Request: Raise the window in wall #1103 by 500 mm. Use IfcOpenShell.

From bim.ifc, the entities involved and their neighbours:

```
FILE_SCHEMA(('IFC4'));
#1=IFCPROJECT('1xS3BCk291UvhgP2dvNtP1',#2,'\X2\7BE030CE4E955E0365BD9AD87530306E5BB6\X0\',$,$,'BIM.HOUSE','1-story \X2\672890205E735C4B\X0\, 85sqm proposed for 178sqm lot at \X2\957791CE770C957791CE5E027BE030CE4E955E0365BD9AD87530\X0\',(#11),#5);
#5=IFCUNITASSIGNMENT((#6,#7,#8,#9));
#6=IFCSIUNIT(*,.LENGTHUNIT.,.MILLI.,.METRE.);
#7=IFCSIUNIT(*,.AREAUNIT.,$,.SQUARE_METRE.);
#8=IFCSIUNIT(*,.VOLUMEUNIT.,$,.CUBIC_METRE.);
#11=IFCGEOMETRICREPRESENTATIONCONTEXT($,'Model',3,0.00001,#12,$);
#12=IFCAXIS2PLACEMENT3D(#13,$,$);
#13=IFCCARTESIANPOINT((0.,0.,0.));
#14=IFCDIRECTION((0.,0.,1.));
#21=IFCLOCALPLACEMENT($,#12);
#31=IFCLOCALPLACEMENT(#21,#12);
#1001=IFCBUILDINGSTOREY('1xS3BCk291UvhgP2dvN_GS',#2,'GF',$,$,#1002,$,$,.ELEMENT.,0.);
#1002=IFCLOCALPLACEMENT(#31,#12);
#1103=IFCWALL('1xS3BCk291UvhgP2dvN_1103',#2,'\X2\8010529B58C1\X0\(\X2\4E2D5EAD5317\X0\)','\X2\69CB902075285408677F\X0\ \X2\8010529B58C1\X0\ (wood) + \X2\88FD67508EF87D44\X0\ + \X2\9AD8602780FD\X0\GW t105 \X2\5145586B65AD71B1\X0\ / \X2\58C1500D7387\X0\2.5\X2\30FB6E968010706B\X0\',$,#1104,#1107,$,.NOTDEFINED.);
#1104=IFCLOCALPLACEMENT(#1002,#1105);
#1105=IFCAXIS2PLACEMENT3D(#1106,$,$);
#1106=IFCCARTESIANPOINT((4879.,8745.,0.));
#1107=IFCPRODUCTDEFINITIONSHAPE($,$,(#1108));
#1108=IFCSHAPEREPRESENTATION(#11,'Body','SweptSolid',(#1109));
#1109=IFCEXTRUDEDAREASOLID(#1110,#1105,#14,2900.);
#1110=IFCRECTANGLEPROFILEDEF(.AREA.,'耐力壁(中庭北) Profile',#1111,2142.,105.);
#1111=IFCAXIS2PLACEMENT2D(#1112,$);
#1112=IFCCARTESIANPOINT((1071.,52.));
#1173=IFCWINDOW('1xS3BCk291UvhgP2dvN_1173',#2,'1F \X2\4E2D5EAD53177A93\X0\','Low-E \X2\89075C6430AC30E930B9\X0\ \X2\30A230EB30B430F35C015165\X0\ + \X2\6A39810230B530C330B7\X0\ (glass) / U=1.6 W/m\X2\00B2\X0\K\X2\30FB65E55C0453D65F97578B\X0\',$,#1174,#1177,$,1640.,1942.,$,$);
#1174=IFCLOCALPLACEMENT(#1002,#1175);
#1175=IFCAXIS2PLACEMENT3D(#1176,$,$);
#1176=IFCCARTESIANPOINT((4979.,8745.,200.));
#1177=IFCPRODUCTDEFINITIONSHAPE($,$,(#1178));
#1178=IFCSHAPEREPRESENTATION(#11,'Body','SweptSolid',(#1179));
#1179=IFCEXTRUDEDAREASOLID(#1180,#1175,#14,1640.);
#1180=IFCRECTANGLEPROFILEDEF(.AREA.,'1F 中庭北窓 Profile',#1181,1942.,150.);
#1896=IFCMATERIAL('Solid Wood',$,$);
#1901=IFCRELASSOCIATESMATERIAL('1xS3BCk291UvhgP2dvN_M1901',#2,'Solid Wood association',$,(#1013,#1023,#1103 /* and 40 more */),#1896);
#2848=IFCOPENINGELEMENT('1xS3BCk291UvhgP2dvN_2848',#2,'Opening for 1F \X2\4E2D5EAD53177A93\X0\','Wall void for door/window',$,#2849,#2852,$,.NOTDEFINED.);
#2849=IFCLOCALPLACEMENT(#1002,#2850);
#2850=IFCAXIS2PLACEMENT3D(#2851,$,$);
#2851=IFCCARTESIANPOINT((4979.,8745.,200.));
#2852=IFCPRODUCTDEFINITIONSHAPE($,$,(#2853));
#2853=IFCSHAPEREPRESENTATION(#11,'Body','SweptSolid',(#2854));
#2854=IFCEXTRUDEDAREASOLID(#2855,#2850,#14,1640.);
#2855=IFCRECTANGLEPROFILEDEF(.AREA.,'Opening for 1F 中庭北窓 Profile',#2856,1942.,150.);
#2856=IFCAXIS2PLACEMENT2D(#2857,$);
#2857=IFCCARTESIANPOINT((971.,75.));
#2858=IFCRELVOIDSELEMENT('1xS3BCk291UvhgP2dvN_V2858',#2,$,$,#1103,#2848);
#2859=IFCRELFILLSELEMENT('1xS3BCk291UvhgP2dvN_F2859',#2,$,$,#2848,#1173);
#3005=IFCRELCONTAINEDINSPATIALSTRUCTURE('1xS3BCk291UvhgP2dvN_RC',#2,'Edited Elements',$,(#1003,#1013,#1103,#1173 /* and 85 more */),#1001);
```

```python
import numpy as np
import ifcopenshell
import ifcopenshell.api.geometry
import ifcopenshell.util.placement
import ifcopenshell.util.unit

model = ifcopenshell.open("bim.ifc")
unit_scale = ifcopenshell.util.unit.calculate_unit_scale(model)

window = model.by_id(1173)
opening = window.FillsVoids[0].RelatingOpeningElement
dz = 0.5 / unit_scale

shift = np.array([0.0, 0.0, dz])
# The window is not placed relative to its opening, so move both.
for product in (opening, window):
    matrix = ifcopenshell.util.placement.get_local_placement(product.ObjectPlacement)
    matrix[:3, 3] += shift
    ifcopenshell.api.geometry.edit_object_placement(model, product=product, matrix=matrix, is_si=False)

print(f"moved by {dz * unit_scale:+.3f} m")

model.write("bim-out.ifc")
```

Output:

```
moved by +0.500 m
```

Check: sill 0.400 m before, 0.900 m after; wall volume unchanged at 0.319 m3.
